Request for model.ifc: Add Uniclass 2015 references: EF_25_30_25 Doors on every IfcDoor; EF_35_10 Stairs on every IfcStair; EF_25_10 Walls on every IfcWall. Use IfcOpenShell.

First a look at what the model holds.

```python
import ifcopenshell

model = ifcopenshell.open("model.ifc")
print(model.schema)
print("classifications:", [c.Name for c in model.by_type("IfcClassification")])
for ifc_class in ("IfcDoor", "IfcRoof", "IfcStair", "IfcWall", "IfcWindow"):
    print(ifc_class, len(model.by_type(ifc_class)))
```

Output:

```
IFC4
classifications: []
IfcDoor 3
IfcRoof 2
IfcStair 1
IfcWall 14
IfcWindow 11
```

```python
import ifcopenshell
import ifcopenshell.api.classification

model = ifcopenshell.open("model.ifc")

system = ifcopenshell.api.classification.add_classification(model, classification="Uniclass 2015")

codes = {
    "IfcDoor": ("EF_25_30_25", "Doors"),
    "IfcStair": ("EF_35_10", "Stairs"),
    "IfcWall": ("EF_25_10", "Walls"),
}
for ifc_class, (code, name) in codes.items():
    products = model.by_type(ifc_class)
    ifcopenshell.api.classification.add_reference(
        model, products=products, classification=system, identification=code, name=name
    )
    print(code, len(products))

model.write("model_v2.ifc")
```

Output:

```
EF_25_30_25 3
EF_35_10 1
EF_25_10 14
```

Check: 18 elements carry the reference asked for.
